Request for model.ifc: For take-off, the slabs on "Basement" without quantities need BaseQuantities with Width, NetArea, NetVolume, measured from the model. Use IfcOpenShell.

First a look at what the model holds.

```python
import ifcopenshell
import ifcopenshell.util.element
import ifcopenshell.util.unit

model = ifcopenshell.open("model.ifc")
print(model.schema)
for unit_type in ("LENGTHUNIT", "AREAUNIT", "VOLUMEUNIT"):
    print(unit_type, ifcopenshell.util.unit.calculate_unit_scale(model, unit_type))
storey = next(s for s in model.by_type("IfcBuildingStorey") if s.Name == "Basement")
slabs = [e for e in ifcopenshell.util.element.get_decomposition(storey) if e.is_a("IfcSlab")]
for e in sorted(slabs, key=lambda e: e.id()):
    print(e.id(), e.is_a(), e.Name, list(ifcopenshell.util.element.get_psets(e, qtos_only=True)), sep=" | ")
```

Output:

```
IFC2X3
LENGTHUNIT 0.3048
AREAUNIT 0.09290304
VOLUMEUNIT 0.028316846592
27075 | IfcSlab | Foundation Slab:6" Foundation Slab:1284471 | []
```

```python
import ifcopenshell
import ifcopenshell.api.pset
import ifcopenshell.geom
import ifcopenshell.util.element
import ifcopenshell.util.shape
import ifcopenshell.util.unit

model = ifcopenshell.open("model.ifc")
unit_scale = ifcopenshell.util.unit.calculate_unit_scale(model)
area_scale = ifcopenshell.util.unit.calculate_unit_scale(model, "AREAUNIT")
volume_scale = ifcopenshell.util.unit.calculate_unit_scale(model, "VOLUMEUNIT")
settings = ifcopenshell.geom.settings()

storey = next(s for s in model.by_type("IfcBuildingStorey") if s.Name == "Basement")
slabs = [e for e in ifcopenshell.util.element.get_decomposition(storey) if e.is_a("IfcSlab")]

for e in sorted(slabs, key=lambda e: e.id()):
    if ifcopenshell.util.element.get_psets(e, qtos_only=True, should_inherit=False):
        continue
    # Geometry comes back in metres, in the element's own axes.
    shape = ifcopenshell.geom.create_shape(settings, e)
    values = {
        "Width": ifcopenshell.util.shape.get_z(shape.geometry) / unit_scale,
        "NetArea": ifcopenshell.util.shape.get_footprint_area(shape.geometry) / area_scale,
        "NetVolume": ifcopenshell.util.shape.get_volume(shape.geometry) / volume_scale,
    }
    qto = ifcopenshell.api.pset.add_qto(model, product=e, name="BaseQuantities")
    ifcopenshell.api.pset.edit_qto(model, qto=qto, properties=values)
    print(e.id(), {k: round(v, 3) for k, v in values.items()})

model.write("model_v2.ifc")
```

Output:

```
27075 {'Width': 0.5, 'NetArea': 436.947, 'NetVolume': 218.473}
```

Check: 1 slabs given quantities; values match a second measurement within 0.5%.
